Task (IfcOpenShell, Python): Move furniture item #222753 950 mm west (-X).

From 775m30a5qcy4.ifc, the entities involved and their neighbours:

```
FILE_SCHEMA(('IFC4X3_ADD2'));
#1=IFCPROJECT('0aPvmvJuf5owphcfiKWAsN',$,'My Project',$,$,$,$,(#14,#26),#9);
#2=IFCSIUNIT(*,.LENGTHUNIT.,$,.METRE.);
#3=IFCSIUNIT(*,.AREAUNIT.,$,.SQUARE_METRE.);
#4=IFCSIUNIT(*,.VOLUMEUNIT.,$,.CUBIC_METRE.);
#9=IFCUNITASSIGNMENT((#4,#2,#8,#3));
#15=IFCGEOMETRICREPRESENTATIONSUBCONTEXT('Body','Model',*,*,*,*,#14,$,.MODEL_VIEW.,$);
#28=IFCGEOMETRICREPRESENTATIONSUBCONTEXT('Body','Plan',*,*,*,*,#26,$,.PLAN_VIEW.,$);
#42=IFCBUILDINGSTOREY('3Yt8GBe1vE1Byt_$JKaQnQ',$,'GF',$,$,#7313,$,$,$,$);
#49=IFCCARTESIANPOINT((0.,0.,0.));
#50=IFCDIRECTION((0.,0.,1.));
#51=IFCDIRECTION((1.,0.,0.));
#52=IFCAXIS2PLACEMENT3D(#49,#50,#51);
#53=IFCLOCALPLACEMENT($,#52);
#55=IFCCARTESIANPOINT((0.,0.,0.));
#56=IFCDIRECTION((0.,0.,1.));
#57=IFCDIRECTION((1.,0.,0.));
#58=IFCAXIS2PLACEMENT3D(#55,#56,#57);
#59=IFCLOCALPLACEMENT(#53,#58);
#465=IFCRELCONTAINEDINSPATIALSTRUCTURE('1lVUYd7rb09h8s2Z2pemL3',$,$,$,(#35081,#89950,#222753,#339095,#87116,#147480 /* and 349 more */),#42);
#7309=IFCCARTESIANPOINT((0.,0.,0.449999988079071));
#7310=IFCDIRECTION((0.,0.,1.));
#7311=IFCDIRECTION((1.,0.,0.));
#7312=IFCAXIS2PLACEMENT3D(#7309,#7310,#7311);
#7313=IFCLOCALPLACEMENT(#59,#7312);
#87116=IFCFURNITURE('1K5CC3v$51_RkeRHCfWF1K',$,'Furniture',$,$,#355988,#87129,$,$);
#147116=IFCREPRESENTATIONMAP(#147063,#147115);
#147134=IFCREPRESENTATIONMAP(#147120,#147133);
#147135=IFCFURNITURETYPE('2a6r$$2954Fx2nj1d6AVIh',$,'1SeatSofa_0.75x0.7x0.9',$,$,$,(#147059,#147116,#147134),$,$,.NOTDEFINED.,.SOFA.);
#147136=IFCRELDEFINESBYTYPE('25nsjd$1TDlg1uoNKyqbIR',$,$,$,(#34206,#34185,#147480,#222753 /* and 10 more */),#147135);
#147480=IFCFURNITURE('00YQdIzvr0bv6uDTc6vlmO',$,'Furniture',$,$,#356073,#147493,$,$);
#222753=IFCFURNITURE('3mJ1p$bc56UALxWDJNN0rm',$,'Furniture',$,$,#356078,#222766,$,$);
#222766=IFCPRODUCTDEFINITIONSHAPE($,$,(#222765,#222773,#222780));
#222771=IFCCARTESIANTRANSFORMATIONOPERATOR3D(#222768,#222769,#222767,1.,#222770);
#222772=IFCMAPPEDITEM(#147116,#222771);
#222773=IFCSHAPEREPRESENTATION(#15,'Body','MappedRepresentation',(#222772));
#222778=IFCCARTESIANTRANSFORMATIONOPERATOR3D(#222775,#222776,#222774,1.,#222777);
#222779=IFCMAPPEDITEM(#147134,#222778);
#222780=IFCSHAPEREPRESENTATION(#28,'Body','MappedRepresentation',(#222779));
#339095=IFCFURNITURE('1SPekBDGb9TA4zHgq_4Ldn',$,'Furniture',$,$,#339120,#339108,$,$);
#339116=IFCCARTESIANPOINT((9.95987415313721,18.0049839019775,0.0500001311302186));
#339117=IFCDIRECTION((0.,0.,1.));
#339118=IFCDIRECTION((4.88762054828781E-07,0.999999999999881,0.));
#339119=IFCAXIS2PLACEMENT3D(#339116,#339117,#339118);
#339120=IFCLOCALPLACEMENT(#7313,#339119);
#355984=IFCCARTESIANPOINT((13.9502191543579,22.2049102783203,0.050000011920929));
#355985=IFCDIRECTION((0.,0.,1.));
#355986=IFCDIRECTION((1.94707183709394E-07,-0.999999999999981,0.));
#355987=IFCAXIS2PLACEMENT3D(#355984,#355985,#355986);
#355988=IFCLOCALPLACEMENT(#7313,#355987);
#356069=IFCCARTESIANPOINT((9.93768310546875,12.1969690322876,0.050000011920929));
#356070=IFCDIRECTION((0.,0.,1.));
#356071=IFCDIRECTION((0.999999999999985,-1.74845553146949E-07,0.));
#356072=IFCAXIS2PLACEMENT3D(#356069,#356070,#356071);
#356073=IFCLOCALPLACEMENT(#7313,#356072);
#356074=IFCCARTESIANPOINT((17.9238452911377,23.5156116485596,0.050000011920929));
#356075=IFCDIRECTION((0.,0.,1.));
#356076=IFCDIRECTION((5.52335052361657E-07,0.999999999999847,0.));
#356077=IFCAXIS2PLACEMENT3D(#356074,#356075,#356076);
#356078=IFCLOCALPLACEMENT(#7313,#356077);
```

```python
import ifcopenshell
import ifcopenshell.api.geometry
import ifcopenshell.util.placement
import ifcopenshell.util.unit

model = ifcopenshell.open("775m30a5qcy4.ifc")
unit_scale = ifcopenshell.util.unit.calculate_unit_scale(model)

item = model.by_guid("3mJ1p$bc56UALxWDJNN0rm")
matrix = ifcopenshell.util.placement.get_local_placement(item.ObjectPlacement)
matrix[0, 3] -= 0.95 / unit_scale
ifcopenshell.api.geometry.edit_object_placement(model, product=item, matrix=matrix, is_si=False)

print(ifcopenshell.util.placement.get_local_placement(item.ObjectPlacement).round(3) + 0.0)

model.write("775m30a5qcy4_updated.ifc")
```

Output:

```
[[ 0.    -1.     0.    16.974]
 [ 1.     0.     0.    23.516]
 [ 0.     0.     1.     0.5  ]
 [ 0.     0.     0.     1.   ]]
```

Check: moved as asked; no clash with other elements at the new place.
